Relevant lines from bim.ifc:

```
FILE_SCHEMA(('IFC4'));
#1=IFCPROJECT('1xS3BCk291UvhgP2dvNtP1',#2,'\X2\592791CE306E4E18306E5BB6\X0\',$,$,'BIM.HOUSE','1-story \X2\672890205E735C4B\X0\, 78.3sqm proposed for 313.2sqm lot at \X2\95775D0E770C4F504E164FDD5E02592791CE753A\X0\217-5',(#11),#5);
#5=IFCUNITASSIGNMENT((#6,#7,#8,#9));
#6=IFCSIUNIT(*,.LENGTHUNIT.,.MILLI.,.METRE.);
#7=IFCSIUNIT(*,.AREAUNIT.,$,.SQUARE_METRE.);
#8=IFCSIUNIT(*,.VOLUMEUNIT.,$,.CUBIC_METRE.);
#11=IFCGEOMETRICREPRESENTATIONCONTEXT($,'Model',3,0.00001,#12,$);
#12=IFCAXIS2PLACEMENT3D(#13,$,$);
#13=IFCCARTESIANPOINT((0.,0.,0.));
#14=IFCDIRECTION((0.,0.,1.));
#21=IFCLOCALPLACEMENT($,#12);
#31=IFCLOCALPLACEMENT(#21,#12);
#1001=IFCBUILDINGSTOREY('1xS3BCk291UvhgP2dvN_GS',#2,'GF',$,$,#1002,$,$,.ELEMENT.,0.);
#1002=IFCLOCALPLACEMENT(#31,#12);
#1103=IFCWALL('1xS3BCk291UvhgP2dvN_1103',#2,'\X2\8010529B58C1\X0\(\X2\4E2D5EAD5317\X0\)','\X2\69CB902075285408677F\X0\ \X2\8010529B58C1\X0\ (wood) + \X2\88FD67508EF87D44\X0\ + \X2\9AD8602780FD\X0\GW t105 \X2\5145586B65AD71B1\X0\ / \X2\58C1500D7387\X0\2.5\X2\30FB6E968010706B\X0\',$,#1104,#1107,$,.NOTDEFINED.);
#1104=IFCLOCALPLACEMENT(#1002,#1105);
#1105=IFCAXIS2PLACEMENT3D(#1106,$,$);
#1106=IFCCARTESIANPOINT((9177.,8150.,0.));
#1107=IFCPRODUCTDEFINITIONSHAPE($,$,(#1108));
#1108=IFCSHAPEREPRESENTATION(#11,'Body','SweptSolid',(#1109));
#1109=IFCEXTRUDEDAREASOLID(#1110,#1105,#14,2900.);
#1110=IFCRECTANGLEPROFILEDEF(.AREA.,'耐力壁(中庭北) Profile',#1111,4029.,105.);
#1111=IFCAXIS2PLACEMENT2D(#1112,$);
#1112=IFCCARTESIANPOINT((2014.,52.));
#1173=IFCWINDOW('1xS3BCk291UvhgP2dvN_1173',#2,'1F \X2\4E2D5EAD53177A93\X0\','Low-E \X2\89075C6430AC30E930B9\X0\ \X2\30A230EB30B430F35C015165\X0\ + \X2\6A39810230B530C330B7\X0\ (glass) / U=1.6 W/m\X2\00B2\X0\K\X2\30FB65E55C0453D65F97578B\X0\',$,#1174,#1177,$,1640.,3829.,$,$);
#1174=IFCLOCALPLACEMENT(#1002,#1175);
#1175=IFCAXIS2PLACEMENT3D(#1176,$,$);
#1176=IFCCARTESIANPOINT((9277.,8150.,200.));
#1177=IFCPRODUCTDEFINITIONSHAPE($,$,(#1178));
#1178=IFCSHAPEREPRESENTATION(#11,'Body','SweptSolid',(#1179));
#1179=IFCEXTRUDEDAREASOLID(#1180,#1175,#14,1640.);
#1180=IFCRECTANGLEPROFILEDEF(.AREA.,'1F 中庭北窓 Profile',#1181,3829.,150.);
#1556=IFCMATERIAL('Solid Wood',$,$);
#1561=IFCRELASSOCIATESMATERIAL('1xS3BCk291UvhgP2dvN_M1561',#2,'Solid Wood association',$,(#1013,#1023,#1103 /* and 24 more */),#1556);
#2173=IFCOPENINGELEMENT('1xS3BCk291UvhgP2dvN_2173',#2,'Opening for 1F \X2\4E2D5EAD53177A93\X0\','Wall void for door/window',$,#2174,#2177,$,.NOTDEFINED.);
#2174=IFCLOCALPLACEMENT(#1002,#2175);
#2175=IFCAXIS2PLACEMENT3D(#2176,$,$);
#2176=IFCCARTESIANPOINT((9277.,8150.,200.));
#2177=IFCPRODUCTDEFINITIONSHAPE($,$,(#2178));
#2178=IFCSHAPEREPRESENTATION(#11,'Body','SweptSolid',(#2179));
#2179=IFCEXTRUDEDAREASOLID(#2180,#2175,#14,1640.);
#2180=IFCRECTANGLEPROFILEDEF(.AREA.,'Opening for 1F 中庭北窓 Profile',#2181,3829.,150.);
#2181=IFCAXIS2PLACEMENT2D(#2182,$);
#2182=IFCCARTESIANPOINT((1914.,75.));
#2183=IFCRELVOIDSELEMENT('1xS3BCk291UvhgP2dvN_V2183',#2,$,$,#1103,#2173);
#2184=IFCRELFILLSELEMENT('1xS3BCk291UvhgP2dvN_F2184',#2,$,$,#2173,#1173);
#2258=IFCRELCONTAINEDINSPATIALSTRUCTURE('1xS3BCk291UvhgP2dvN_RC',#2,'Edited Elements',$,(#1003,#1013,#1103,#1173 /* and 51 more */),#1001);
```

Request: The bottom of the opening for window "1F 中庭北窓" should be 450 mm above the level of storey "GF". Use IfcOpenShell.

```python
import numpy as np
import ifcopenshell
import ifcopenshell.api.geometry
import ifcopenshell.geom
import ifcopenshell.util.element
import ifcopenshell.util.placement
import ifcopenshell.util.shape
import ifcopenshell.util.unit

model = ifcopenshell.open("bim.ifc")
unit_scale = ifcopenshell.util.unit.calculate_unit_scale(model)

window = model.by_id(1173)
opening = window.FillsVoids[0].RelatingOpeningElement
storey = ifcopenshell.util.element.get_container(window, ifc_class="IfcBuildingStorey")
level = ifcopenshell.util.placement.get_local_placement(storey.ObjectPlacement)[2, 3]

# The opening's origin need not be at the sill, so measure its lowest point.
shape = ifcopenshell.geom.create_shape(ifcopenshell.geom.settings(), opening)
bottom = ifcopenshell.util.shape.get_shape_bottom_elevation(shape, shape.geometry) / unit_scale
dz = level + 450.0 - bottom

shift = np.array([0.0, 0.0, dz])
# The window is not placed relative to its opening, so move both.
for product in (opening, window):
    matrix = ifcopenshell.util.placement.get_local_placement(product.ObjectPlacement)
    matrix[:3, 3] += shift
    ifcopenshell.api.geometry.edit_object_placement(model, product=product, matrix=matrix, is_si=False)

print(f"moved by {dz * unit_scale:+.3f} m")

model.write("bim-out.ifc")
```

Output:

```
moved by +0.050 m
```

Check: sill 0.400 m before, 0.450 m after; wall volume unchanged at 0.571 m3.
